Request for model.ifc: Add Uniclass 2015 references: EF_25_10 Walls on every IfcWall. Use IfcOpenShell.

First a look at what the model holds.

```python
import ifcopenshell

model = ifcopenshell.open("model.ifc")
print(model.schema)
print("classifications:", [c.Name for c in model.by_type("IfcClassification")])
for ifc_class in ("IfcDoor", "IfcRoof", "IfcStair", "IfcWall", "IfcWindow"):
    print(ifc_class, len(model.by_type(ifc_class)))
```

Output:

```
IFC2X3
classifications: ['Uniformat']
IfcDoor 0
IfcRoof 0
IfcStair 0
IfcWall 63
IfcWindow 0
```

```python
import ifcopenshell
import ifcopenshell.api.classification

model = ifcopenshell.open("model.ifc")

# IFC2X3 requires Source and Edition and has no link from the project to the system.
system = model.create_entity("IfcClassification", Source="NBS", Edition="2015", Name="Uniclass 2015")

codes = {
    "IfcWall": ("EF_25_10", "Walls"),
}
for ifc_class, (code, name) in codes.items():
    products = model.by_type(ifc_class)
    ifcopenshell.api.classification.add_reference(
        model, products=products, classification=system, identification=code, name=name
    )
    print(code, len(products))

model.write("model-out.ifc")
```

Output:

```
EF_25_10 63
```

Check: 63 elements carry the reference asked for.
